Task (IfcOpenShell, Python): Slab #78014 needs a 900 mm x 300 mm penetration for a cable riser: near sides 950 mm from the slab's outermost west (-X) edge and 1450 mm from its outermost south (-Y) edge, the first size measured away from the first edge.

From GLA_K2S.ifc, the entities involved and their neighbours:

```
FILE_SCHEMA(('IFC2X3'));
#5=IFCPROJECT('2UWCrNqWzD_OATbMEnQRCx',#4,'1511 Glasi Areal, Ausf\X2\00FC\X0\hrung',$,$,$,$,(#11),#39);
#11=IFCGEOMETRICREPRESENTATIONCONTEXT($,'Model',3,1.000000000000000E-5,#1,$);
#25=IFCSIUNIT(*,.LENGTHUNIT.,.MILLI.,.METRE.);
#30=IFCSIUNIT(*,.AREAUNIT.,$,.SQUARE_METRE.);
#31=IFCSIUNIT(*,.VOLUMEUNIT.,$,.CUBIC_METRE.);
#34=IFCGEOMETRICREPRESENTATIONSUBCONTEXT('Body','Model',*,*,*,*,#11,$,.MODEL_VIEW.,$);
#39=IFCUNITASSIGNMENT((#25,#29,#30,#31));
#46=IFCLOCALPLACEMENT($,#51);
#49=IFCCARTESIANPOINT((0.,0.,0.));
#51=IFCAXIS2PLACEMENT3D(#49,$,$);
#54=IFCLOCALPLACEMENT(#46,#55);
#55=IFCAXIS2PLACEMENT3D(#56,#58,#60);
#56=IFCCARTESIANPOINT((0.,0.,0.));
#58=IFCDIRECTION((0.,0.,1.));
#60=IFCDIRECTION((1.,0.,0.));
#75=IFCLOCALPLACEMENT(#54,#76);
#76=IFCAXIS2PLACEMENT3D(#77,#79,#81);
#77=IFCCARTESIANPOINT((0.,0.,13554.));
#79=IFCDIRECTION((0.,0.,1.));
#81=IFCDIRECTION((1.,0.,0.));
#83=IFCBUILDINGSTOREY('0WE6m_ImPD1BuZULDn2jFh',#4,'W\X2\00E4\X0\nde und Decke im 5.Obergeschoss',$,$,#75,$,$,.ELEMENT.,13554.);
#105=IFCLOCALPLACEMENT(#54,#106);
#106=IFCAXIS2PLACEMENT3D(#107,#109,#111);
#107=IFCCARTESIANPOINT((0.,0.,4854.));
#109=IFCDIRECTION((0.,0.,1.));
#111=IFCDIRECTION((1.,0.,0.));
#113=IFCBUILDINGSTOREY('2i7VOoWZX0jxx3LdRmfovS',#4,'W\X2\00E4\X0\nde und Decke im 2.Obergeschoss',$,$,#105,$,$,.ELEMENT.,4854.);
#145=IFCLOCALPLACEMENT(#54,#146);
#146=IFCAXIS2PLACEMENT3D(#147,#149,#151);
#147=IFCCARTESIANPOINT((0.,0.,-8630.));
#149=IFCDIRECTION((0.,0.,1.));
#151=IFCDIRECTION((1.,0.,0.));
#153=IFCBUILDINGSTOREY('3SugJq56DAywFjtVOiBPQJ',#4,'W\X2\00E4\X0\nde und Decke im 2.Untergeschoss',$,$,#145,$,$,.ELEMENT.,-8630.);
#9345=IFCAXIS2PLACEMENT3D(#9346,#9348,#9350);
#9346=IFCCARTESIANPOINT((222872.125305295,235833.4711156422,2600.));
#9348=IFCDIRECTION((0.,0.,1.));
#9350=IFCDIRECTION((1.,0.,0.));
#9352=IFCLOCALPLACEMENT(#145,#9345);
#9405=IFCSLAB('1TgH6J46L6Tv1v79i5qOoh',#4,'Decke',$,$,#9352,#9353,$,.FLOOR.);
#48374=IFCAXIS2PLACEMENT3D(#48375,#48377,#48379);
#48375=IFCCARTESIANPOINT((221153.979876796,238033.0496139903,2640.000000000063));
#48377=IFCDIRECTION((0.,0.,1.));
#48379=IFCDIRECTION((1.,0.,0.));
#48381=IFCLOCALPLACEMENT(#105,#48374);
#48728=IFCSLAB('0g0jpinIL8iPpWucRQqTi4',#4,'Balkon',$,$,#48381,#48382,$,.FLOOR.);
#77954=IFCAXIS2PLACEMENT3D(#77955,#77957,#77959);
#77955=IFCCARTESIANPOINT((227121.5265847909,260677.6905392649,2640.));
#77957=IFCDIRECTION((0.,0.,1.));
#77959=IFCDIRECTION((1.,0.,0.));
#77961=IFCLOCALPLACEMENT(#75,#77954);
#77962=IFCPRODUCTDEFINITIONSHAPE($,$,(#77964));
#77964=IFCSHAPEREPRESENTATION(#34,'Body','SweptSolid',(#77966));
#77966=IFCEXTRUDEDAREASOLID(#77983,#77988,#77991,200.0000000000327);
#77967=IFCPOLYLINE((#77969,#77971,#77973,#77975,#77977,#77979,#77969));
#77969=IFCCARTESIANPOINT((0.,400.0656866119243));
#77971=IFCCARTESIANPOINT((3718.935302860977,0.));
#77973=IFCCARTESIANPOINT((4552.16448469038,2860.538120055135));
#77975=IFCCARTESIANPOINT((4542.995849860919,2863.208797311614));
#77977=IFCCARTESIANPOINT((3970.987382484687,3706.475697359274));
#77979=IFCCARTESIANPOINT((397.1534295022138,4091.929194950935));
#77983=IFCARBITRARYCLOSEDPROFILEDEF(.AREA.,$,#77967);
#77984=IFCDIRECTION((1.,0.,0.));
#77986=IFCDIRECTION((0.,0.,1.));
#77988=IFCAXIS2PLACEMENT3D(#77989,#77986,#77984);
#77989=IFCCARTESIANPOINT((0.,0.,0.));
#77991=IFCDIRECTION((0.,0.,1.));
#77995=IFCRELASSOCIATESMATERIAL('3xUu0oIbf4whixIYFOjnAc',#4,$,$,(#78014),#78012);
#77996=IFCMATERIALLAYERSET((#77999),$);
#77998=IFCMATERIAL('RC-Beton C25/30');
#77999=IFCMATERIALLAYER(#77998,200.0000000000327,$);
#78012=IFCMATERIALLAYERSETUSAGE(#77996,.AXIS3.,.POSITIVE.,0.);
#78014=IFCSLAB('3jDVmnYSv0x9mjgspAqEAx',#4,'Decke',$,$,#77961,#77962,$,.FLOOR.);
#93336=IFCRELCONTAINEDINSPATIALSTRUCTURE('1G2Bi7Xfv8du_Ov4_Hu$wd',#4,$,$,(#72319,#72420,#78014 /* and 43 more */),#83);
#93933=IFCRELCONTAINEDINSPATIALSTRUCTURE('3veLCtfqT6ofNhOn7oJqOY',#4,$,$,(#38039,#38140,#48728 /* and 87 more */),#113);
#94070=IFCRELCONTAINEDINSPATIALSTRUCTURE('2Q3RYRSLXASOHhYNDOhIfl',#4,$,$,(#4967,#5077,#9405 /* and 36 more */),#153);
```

```python
import numpy as np
import ifcopenshell
import ifcopenshell.api.feature
import ifcopenshell.api.geometry
import ifcopenshell.api.root
import ifcopenshell.geom
import ifcopenshell.util.placement
import ifcopenshell.util.representation
import ifcopenshell.util.shape
import ifcopenshell.util.unit

model = ifcopenshell.open("GLA_K2S.ifc")
unit_scale = ifcopenshell.util.unit.calculate_unit_scale(model)
settings = ifcopenshell.geom.settings()


def volume(element):
    """Net volume in cubic metres, openings subtracted."""
    shape = ifcopenshell.geom.create_shape(settings, element)
    return ifcopenshell.util.shape.get_volume(shape.geometry)


slab = model.by_guid("3jDVmnYSv0x9mjgspAqEAx")
before = volume(slab)

# Extent in the slab's own axes, in metres. The edges named are its -X and -Y sides.
slab_shape = ifcopenshell.geom.create_shape(settings, slab)
vertices = ifcopenshell.util.shape.get_vertices(slab_shape.geometry)
x_min, y_min, bottom = vertices.min(axis=0)
top = vertices[:, 2].max()

opening = ifcopenshell.api.root.create_entity(model, ifc_class="IfcOpeningElement", name="Cable riser opening")
context = ifcopenshell.util.representation.get_context(model, "Model", "Body", "MODEL_VIEW")
width, depth = 0.9, 0.3
outline = [(0.0, 0.0), (width, 0.0), (width, depth), (0.0, depth), (0.0, 0.0)]
# Overshoot both faces by 50 mm so the cut is clean.
shape = ifcopenshell.api.geometry.add_slab_representation(
    model, context=context, depth=top - bottom + 0.1, polyline=outline
)
ifcopenshell.api.geometry.assign_representation(model, product=opening, representation=shape)

matrix = ifcopenshell.util.placement.get_local_placement(slab.ObjectPlacement)
matrix[:, 3] = matrix @ np.append(np.array([x_min + 0.95, y_min + 1.45, bottom - 0.05]) / unit_scale, 1.0)
ifcopenshell.api.geometry.edit_object_placement(model, product=opening, matrix=matrix, is_si=False)
ifcopenshell.api.feature.add_feature(model, feature=opening, element=slab)

after = volume(slab)

print(f"slab volume {before:.3f} -> {after:.3f} m3")

model.write("GLA_K2S_v2.ifc")
```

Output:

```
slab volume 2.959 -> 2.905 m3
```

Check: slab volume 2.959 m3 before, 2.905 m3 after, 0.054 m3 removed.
